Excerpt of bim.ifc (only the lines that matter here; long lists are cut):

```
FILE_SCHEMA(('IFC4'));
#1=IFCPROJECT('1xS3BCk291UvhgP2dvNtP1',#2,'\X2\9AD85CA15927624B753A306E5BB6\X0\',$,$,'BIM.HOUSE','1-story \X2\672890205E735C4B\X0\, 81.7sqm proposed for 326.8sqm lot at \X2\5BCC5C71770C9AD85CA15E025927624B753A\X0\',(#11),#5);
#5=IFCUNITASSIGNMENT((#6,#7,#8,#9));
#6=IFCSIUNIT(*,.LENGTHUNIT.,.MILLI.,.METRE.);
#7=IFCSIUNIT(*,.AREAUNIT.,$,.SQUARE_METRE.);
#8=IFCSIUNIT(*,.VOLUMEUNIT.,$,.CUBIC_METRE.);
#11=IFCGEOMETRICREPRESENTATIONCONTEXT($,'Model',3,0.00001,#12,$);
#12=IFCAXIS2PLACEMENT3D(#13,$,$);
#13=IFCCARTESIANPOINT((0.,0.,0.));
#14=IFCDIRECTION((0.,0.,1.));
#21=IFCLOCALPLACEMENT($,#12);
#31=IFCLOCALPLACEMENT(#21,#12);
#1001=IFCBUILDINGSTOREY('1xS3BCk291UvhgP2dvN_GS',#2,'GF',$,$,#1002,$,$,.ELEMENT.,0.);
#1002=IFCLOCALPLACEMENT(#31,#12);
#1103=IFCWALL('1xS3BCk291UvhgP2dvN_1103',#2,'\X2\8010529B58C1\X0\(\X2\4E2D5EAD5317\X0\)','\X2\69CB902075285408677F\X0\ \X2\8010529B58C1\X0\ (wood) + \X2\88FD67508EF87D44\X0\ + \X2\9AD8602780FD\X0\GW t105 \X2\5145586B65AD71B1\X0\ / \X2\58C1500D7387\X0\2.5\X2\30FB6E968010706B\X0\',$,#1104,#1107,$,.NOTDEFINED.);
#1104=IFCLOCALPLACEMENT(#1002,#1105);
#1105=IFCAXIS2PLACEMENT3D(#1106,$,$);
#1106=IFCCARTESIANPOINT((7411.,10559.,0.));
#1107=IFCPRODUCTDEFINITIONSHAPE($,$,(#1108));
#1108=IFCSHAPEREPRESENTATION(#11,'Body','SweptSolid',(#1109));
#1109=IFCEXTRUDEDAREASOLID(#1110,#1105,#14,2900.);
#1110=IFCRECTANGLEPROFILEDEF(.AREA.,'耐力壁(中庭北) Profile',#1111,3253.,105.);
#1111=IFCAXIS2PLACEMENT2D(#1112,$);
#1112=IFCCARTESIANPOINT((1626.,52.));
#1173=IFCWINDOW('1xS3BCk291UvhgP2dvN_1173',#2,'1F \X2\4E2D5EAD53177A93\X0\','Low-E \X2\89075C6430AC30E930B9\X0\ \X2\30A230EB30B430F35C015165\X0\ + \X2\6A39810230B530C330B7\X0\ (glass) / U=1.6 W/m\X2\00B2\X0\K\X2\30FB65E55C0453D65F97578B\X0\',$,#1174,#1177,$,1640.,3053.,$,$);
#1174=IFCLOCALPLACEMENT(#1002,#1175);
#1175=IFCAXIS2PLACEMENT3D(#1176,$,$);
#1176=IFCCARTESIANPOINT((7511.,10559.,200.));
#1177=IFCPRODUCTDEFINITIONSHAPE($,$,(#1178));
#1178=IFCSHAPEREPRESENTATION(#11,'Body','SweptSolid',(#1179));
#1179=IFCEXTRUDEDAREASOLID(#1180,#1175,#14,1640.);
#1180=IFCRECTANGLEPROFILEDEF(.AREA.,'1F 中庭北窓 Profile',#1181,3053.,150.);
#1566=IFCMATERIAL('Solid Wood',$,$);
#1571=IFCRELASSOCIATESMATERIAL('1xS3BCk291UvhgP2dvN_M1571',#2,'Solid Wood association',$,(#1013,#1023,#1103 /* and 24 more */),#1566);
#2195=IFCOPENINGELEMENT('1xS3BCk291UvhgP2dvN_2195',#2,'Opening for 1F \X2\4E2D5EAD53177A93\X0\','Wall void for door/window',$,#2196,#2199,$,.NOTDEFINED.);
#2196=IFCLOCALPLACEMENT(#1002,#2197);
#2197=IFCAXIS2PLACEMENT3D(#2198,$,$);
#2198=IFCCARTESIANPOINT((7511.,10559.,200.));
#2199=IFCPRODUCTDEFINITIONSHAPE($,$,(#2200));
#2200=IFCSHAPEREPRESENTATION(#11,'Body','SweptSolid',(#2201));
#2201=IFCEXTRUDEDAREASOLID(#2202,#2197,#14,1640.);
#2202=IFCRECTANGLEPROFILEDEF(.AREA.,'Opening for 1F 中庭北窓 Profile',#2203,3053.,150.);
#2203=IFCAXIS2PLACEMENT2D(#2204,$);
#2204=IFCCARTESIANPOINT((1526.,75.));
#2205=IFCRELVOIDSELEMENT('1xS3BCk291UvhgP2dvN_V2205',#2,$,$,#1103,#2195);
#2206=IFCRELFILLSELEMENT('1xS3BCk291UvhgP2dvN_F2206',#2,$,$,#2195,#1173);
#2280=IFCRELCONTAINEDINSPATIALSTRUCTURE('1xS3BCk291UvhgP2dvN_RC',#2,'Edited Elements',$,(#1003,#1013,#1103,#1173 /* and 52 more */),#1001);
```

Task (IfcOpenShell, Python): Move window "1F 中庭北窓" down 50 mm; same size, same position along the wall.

```python
import numpy as np
import ifcopenshell
import ifcopenshell.api.geometry
import ifcopenshell.util.placement
import ifcopenshell.util.unit

model = ifcopenshell.open("bim.ifc")
unit_scale = ifcopenshell.util.unit.calculate_unit_scale(model)

window = model.by_guid("1xS3BCk291UvhgP2dvN_1173")
opening = window.FillsVoids[0].RelatingOpeningElement
dz = -0.05 / unit_scale

shift = np.array([0.0, 0.0, dz])
# The window is not placed relative to its opening, so move both.
for product in (opening, window):
    matrix = ifcopenshell.util.placement.get_local_placement(product.ObjectPlacement)
    matrix[:3, 3] += shift
    ifcopenshell.api.geometry.edit_object_placement(model, product=product, matrix=matrix, is_si=False)

print(f"moved by {dz * unit_scale:+.3f} m")

model.write("bim-out.ifc")
```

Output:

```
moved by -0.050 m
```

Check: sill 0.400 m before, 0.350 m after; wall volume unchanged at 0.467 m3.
